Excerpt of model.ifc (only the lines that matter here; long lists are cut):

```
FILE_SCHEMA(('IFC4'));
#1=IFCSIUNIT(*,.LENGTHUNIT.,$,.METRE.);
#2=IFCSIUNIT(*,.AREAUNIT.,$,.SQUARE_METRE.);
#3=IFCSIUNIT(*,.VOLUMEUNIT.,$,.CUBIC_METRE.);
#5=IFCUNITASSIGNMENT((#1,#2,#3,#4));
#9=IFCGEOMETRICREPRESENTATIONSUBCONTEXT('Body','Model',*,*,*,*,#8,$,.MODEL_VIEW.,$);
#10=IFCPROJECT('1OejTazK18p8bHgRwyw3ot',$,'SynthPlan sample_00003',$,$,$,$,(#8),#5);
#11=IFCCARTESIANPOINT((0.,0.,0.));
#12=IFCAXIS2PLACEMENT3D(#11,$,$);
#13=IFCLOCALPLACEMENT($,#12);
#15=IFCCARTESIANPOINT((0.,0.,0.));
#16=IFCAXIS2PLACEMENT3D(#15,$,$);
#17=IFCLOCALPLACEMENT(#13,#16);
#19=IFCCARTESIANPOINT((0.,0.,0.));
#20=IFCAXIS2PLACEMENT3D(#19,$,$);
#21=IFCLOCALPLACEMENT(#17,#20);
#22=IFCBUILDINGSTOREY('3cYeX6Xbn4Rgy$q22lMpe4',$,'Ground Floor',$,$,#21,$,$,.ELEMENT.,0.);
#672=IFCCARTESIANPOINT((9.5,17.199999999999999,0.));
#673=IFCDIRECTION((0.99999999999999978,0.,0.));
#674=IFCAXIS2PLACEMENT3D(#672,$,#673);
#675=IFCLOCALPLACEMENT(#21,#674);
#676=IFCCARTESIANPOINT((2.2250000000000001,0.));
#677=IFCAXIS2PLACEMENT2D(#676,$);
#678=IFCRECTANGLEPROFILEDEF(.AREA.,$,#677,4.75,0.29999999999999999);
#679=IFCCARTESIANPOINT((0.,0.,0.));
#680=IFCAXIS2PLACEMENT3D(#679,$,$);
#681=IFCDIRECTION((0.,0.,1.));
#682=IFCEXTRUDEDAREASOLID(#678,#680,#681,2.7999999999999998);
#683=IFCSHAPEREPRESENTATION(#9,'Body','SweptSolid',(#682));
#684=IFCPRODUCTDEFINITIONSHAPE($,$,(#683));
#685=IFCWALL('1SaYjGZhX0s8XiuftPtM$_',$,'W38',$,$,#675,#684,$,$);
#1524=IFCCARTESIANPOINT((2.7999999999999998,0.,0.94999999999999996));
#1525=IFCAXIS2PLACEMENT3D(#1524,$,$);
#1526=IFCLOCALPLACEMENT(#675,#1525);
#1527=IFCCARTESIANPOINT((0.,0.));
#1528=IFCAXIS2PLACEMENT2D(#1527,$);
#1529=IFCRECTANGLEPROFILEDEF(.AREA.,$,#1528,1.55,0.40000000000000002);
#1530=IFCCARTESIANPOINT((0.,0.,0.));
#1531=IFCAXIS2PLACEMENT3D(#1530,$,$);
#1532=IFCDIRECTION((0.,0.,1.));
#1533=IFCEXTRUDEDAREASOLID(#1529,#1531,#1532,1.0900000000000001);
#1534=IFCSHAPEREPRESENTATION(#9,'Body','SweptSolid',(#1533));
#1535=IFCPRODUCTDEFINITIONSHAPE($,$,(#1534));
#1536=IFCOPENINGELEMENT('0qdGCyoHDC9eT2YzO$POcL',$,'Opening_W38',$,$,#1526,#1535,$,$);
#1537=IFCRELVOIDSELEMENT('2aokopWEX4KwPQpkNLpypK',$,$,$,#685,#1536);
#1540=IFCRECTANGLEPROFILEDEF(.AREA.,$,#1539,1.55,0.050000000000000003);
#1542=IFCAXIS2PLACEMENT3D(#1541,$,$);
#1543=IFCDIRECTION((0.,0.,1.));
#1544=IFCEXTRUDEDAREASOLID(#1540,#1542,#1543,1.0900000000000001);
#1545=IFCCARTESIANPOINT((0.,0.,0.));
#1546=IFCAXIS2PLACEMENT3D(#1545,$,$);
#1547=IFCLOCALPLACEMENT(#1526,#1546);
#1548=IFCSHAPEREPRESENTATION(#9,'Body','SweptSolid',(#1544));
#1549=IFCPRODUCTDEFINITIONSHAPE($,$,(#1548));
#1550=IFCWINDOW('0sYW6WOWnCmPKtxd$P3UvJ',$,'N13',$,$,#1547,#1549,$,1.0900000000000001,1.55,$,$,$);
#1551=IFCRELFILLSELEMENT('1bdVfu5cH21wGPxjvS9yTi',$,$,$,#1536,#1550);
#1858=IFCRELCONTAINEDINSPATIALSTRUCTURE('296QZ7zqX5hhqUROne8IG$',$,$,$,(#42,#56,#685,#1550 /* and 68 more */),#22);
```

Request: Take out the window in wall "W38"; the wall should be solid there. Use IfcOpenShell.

```python
import ifcopenshell
import ifcopenshell.api.feature
import ifcopenshell.api.root
import ifcopenshell.geom
import ifcopenshell.util.shape

model = ifcopenshell.open("model.ifc")
settings = ifcopenshell.geom.settings()


def volume(element):
    """Net volume in cubic metres, openings subtracted."""
    shape = ifcopenshell.geom.create_shape(settings, element)
    return ifcopenshell.util.shape.get_volume(shape.geometry)


window = model.by_guid("0sYW6WOWnCmPKtxd$P3UvJ")
opening = window.FillsVoids[0].RelatingOpeningElement
wall = opening.VoidsElements[0].RelatingBuildingElement
before = volume(wall)

ifcopenshell.api.root.remove_product(model, product=window)
ifcopenshell.api.feature.remove_feature(model, feature=opening)

after = volume(wall)

print(f"wall volume {before:.3f} -> {after:.3f} m3")

model.write("model_rev.ifc")
```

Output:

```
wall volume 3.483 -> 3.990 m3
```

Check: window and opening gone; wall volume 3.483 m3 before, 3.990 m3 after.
